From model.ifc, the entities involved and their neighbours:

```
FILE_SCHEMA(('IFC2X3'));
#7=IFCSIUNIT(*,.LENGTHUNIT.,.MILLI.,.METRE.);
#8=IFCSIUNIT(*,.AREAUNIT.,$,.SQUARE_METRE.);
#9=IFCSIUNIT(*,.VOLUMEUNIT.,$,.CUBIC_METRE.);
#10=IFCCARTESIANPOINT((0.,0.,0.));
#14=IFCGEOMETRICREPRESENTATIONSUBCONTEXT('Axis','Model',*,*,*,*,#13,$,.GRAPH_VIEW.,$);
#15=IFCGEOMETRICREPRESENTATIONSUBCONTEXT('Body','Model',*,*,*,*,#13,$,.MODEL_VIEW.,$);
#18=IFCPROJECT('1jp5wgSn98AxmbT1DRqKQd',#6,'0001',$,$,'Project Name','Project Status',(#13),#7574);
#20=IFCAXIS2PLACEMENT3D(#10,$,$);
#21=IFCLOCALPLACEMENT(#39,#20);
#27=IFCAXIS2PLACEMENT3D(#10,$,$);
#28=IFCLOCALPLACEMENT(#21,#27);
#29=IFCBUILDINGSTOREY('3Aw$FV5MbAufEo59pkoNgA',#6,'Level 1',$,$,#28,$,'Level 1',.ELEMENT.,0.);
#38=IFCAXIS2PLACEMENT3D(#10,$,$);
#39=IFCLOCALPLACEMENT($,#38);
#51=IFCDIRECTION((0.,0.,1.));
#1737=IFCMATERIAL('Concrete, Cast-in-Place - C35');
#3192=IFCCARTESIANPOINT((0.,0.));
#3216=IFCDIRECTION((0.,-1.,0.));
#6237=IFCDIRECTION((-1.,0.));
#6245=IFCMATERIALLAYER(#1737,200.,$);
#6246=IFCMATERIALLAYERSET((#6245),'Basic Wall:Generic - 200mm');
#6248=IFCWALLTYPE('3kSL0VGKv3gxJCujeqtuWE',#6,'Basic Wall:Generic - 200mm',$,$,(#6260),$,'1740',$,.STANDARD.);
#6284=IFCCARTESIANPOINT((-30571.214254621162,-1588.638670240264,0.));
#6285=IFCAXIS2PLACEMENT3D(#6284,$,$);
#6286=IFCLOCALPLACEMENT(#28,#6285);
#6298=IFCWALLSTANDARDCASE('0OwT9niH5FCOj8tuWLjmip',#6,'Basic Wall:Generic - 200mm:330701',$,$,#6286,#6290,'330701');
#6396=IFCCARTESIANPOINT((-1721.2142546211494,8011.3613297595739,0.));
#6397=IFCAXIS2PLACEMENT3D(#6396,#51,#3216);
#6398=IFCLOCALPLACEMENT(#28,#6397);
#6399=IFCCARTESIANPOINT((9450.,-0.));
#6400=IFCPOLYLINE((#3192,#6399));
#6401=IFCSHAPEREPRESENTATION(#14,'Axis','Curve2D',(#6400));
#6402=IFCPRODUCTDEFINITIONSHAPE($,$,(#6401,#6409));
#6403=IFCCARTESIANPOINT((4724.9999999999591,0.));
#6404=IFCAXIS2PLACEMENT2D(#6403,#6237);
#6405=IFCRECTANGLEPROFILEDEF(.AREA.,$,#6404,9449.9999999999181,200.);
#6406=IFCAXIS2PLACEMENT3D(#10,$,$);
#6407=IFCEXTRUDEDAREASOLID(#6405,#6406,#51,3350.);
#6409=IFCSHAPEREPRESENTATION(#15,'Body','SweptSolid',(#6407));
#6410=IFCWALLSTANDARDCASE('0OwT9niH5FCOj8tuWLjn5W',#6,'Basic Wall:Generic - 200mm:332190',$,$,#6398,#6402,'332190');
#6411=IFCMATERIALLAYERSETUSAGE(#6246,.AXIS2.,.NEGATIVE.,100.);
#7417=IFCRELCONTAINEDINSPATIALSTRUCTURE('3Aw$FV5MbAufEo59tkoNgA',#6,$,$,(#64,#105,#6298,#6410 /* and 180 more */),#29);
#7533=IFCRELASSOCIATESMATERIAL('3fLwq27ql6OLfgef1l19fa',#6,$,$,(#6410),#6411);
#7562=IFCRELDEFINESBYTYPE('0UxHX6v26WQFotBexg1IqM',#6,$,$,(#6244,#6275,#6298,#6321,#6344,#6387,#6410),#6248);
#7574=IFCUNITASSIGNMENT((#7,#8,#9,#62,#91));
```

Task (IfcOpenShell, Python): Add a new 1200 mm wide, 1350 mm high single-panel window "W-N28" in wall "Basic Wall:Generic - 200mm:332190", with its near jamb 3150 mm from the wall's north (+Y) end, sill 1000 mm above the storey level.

```python
import numpy as np
import ifcopenshell
import ifcopenshell.api.feature
import ifcopenshell.api.geometry
import ifcopenshell.api.root
import ifcopenshell.api.spatial
import ifcopenshell.api.type
import ifcopenshell.geom
import ifcopenshell.util.element
import ifcopenshell.util.placement
import ifcopenshell.util.representation
import ifcopenshell.util.shape
import ifcopenshell.util.unit

model = ifcopenshell.open("model.ifc")
unit_scale = ifcopenshell.util.unit.calculate_unit_scale(model)
settings = ifcopenshell.geom.settings()


def volume(element):
    """Net volume in cubic metres, openings subtracted."""
    shape = ifcopenshell.geom.create_shape(settings, element)
    return ifcopenshell.util.shape.get_volume(shape.geometry)


wall = model.by_guid("0OwT9niH5FCOj8tuWLjn5W")
storey = ifcopenshell.util.element.get_container(wall, ifc_class="IfcBuildingStorey")
context = ifcopenshell.util.representation.get_context(model, "Model", "Body", "MODEL_VIEW")
before = volume(wall)

width, height, from_end, sill = 1.2, 1.35, 3.15, 1  # metres

# The wall runs along its own X axis, and the end named is its -X end.
wall_shape = ifcopenshell.geom.create_shape(settings, wall)
x, y, z = ifcopenshell.util.shape.get_vertices(wall_shape.geometry).T
start = x.min() + from_end
face, thickness = float(y.min()), float(y.max() - y.min())
wall_matrix = ifcopenshell.util.placement.get_local_placement(wall.ObjectPlacement)
level = ifcopenshell.util.placement.get_local_placement(storey.ObjectPlacement)[2, 3]


def in_wall(x, y):
    """Placement at x, y metres in the wall's axes, at sill height."""
    matrix = wall_matrix.copy()
    matrix[:, 3] = wall_matrix @ np.array([x / unit_scale, y / unit_scale, 0.0, 1.0])
    matrix[2, 3] = level + sill / unit_scale
    return matrix


# Opening: a box that overshoots both wall faces by 50 mm.
opening = ifcopenshell.api.root.create_entity(model, ifc_class="IfcOpeningElement")
box = ifcopenshell.api.geometry.add_wall_representation(
    model, context=context, length=width, height=height, thickness=thickness + 0.1
)
ifcopenshell.api.geometry.assign_representation(model, product=opening, representation=box)
ifcopenshell.api.geometry.edit_object_placement(model, product=opening, matrix=in_wall(start, face - 0.05), is_si=False)
ifcopenshell.api.feature.add_feature(model, feature=opening, element=wall)

window = ifcopenshell.api.root.create_entity(model, ifc_class="IfcWindow", name="W-N28")
window.OverallWidth, window.OverallHeight = width / unit_scale, height / unit_scale
body = ifcopenshell.api.geometry.add_window_representation(
    model,
    context=context,
    overall_width=window.OverallWidth,
    overall_height=window.OverallHeight,
    partition_type="SINGLE_PANEL",
)
ifcopenshell.api.geometry.assign_representation(model, product=window, representation=body)
ifcopenshell.api.spatial.assign_container(model, products=[window], relating_structure=storey)
fills = ifcopenshell.api.feature.add_filling(model, opening=opening, element=window)
fills.OwnerHistory = window.OwnerHistory  # required in IFC2X3

# IFC2X3 keeps the operation on the window style.
style = ifcopenshell.api.root.create_entity(model, ifc_class="IfcWindowStyle", name="W-N28")
style.OperationType, style.ConstructionType = "SINGLE_PANEL", "NOTDEFINED"
style.ParameterTakesPrecedence = style.Sizeable = False
ifcopenshell.api.type.assign_type(model, related_objects=[window], relating_type=style)

# Centre the window in the wall's thickness.
ifcopenshell.api.geometry.edit_object_placement(model, product=window, matrix=in_wall(start, face), is_si=False)
window_shape = ifcopenshell.geom.create_shape(settings, window)
depth = ifcopenshell.util.shape.get_vertices(window_shape.geometry)[:, 1]
offset = face + thickness / 2 - (depth.min() + depth.max()) / 2
ifcopenshell.api.geometry.edit_object_placement(model, product=window, matrix=in_wall(start, offset), is_si=False)

after = volume(wall)

print(f"wall volume {before:.3f} -> {after:.3f} m3")

model.write("model-out.ifc")
```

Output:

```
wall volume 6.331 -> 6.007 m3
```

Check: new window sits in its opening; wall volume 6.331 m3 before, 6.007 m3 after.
